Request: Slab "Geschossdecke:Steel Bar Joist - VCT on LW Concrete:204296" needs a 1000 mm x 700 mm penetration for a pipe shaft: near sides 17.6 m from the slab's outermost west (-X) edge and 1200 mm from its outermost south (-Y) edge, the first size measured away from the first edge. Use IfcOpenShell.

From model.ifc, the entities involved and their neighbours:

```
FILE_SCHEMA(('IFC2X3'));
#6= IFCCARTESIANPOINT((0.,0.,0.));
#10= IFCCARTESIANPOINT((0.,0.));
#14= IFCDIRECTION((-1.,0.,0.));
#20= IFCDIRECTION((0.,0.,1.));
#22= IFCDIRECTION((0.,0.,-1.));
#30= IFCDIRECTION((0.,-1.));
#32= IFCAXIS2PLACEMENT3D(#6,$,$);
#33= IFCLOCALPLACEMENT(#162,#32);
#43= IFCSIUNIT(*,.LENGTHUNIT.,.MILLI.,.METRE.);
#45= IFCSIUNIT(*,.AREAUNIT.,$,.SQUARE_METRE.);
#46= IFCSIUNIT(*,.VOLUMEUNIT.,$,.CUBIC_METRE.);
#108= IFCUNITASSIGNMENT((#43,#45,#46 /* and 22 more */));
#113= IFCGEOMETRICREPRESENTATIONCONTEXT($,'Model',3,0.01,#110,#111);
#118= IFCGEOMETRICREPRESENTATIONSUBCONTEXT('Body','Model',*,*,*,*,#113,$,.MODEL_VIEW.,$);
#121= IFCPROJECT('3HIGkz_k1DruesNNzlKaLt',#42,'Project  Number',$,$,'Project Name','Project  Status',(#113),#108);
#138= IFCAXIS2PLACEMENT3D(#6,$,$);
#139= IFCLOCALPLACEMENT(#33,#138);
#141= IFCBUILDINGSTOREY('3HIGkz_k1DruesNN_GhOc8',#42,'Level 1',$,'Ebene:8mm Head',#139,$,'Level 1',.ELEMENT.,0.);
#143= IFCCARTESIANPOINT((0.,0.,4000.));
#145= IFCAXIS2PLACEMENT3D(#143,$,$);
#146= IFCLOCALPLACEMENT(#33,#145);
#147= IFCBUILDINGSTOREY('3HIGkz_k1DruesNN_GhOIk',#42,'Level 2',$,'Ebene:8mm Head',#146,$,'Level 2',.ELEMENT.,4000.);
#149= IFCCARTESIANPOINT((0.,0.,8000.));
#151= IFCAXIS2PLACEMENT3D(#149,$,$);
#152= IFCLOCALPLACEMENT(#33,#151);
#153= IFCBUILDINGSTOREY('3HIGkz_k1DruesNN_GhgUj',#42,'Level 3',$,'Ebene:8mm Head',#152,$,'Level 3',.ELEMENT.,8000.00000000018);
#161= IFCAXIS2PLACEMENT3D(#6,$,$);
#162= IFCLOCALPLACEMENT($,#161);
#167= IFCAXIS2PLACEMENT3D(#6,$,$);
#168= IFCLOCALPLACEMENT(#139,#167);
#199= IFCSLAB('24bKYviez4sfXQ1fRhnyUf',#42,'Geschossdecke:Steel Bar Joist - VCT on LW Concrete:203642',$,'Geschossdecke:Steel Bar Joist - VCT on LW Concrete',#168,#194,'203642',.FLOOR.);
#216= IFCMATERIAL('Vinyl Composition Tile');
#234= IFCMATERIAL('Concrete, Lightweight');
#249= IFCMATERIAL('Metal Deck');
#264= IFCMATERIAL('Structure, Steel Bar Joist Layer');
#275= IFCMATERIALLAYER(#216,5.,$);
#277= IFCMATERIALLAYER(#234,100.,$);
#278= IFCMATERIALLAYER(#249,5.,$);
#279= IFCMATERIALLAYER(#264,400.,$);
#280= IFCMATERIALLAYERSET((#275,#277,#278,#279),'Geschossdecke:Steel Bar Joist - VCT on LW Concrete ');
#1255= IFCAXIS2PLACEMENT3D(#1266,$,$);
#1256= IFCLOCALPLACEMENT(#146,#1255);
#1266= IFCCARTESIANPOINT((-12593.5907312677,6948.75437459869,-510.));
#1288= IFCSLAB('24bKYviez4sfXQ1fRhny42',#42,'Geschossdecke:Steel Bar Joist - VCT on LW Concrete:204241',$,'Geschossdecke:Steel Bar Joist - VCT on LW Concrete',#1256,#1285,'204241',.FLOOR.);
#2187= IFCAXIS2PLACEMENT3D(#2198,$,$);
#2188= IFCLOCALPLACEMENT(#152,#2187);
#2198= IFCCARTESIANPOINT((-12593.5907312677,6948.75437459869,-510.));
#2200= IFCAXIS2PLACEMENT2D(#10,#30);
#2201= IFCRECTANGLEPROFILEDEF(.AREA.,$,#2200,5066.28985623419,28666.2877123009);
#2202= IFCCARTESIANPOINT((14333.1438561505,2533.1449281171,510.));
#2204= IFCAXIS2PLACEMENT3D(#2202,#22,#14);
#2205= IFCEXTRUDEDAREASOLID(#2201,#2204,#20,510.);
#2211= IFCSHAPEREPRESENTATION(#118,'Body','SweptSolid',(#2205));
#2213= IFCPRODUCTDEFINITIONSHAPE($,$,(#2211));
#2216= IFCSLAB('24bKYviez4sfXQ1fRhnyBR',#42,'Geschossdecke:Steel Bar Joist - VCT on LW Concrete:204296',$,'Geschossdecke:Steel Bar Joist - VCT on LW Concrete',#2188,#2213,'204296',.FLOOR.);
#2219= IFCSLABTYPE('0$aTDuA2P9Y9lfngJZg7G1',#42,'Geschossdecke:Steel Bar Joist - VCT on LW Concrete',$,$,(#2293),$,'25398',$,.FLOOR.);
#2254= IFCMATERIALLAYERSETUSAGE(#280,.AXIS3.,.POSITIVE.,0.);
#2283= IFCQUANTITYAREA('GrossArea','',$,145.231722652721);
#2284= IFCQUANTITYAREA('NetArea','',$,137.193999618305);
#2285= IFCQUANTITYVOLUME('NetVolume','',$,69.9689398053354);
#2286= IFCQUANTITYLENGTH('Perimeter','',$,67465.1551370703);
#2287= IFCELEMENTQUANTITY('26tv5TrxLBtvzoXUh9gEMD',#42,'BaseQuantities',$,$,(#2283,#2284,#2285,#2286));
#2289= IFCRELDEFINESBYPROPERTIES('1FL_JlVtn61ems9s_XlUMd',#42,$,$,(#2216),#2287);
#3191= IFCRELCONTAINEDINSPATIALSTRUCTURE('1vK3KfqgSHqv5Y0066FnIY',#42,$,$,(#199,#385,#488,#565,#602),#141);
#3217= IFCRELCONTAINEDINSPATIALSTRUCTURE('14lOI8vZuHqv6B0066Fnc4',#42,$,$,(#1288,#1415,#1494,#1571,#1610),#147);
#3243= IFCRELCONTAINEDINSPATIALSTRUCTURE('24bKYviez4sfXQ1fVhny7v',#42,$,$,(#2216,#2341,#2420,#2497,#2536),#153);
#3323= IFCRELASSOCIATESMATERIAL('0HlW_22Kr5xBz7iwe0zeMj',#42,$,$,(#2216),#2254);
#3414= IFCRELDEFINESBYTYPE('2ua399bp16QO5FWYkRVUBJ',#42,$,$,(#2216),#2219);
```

```python
import numpy as np
import ifcopenshell
import ifcopenshell.api.feature
import ifcopenshell.api.geometry
import ifcopenshell.api.pset
import ifcopenshell.api.root
import ifcopenshell.geom
import ifcopenshell.util.element
import ifcopenshell.util.placement
import ifcopenshell.util.representation
import ifcopenshell.util.shape
import ifcopenshell.util.unit

model = ifcopenshell.open("model.ifc")
unit_scale = ifcopenshell.util.unit.calculate_unit_scale(model)
area_scale = ifcopenshell.util.unit.calculate_unit_scale(model, "AREAUNIT")
volume_scale = ifcopenshell.util.unit.calculate_unit_scale(model, "VOLUMEUNIT")
settings = ifcopenshell.geom.settings()


def volume(element):
    """Net volume in cubic metres, openings subtracted."""
    shape = ifcopenshell.geom.create_shape(settings, element)
    return ifcopenshell.util.shape.get_volume(shape.geometry)


slab = model.by_guid("24bKYviez4sfXQ1fRhnyBR")
before = volume(slab)

# Extent in the slab's own axes, in metres. The edges named are its -X and -Y sides.
slab_shape = ifcopenshell.geom.create_shape(settings, slab)
vertices = ifcopenshell.util.shape.get_vertices(slab_shape.geometry)
x_min, y_min, bottom = vertices.min(axis=0)
top = vertices[:, 2].max()

opening = ifcopenshell.api.root.create_entity(model, ifc_class="IfcOpeningElement", name="Pipe shaft opening")
context = ifcopenshell.util.representation.get_context(model, "Model", "Body", "MODEL_VIEW")
width, depth = 1, 0.7
outline = [(0.0, 0.0), (width, 0.0), (width, depth), (0.0, depth), (0.0, 0.0)]
# Overshoot both faces by 50 mm so the cut is clean.
shape = ifcopenshell.api.geometry.add_slab_representation(
    model, context=context, depth=top - bottom + 0.1, polyline=outline
)
ifcopenshell.api.geometry.assign_representation(model, product=opening, representation=shape)

matrix = ifcopenshell.util.placement.get_local_placement(slab.ObjectPlacement)
matrix[:, 3] = matrix @ np.append(np.array([x_min + 17.6, y_min + 1.2, bottom - 0.05]) / unit_scale, 1.0)
ifcopenshell.api.geometry.edit_object_placement(model, product=opening, matrix=matrix, is_si=False)
ifcopenshell.api.feature.add_feature(model, feature=opening, element=slab)

after = volume(slab)

# Update the slab's stored quantities.
qto = model.by_id(ifcopenshell.util.element.get_pset(slab, "BaseQuantities", should_inherit=False)["id"])
ifcopenshell.api.pset.edit_qto(model, qto=qto, properties={
    "NetArea": after / (top - bottom) / area_scale,
    "NetVolume": after / volume_scale,
})

print(f"slab volume {before:.3f} -> {after:.3f} m3")

model.write("model_edited.ifc")
```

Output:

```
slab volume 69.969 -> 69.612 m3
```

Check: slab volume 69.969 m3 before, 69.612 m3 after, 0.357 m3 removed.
